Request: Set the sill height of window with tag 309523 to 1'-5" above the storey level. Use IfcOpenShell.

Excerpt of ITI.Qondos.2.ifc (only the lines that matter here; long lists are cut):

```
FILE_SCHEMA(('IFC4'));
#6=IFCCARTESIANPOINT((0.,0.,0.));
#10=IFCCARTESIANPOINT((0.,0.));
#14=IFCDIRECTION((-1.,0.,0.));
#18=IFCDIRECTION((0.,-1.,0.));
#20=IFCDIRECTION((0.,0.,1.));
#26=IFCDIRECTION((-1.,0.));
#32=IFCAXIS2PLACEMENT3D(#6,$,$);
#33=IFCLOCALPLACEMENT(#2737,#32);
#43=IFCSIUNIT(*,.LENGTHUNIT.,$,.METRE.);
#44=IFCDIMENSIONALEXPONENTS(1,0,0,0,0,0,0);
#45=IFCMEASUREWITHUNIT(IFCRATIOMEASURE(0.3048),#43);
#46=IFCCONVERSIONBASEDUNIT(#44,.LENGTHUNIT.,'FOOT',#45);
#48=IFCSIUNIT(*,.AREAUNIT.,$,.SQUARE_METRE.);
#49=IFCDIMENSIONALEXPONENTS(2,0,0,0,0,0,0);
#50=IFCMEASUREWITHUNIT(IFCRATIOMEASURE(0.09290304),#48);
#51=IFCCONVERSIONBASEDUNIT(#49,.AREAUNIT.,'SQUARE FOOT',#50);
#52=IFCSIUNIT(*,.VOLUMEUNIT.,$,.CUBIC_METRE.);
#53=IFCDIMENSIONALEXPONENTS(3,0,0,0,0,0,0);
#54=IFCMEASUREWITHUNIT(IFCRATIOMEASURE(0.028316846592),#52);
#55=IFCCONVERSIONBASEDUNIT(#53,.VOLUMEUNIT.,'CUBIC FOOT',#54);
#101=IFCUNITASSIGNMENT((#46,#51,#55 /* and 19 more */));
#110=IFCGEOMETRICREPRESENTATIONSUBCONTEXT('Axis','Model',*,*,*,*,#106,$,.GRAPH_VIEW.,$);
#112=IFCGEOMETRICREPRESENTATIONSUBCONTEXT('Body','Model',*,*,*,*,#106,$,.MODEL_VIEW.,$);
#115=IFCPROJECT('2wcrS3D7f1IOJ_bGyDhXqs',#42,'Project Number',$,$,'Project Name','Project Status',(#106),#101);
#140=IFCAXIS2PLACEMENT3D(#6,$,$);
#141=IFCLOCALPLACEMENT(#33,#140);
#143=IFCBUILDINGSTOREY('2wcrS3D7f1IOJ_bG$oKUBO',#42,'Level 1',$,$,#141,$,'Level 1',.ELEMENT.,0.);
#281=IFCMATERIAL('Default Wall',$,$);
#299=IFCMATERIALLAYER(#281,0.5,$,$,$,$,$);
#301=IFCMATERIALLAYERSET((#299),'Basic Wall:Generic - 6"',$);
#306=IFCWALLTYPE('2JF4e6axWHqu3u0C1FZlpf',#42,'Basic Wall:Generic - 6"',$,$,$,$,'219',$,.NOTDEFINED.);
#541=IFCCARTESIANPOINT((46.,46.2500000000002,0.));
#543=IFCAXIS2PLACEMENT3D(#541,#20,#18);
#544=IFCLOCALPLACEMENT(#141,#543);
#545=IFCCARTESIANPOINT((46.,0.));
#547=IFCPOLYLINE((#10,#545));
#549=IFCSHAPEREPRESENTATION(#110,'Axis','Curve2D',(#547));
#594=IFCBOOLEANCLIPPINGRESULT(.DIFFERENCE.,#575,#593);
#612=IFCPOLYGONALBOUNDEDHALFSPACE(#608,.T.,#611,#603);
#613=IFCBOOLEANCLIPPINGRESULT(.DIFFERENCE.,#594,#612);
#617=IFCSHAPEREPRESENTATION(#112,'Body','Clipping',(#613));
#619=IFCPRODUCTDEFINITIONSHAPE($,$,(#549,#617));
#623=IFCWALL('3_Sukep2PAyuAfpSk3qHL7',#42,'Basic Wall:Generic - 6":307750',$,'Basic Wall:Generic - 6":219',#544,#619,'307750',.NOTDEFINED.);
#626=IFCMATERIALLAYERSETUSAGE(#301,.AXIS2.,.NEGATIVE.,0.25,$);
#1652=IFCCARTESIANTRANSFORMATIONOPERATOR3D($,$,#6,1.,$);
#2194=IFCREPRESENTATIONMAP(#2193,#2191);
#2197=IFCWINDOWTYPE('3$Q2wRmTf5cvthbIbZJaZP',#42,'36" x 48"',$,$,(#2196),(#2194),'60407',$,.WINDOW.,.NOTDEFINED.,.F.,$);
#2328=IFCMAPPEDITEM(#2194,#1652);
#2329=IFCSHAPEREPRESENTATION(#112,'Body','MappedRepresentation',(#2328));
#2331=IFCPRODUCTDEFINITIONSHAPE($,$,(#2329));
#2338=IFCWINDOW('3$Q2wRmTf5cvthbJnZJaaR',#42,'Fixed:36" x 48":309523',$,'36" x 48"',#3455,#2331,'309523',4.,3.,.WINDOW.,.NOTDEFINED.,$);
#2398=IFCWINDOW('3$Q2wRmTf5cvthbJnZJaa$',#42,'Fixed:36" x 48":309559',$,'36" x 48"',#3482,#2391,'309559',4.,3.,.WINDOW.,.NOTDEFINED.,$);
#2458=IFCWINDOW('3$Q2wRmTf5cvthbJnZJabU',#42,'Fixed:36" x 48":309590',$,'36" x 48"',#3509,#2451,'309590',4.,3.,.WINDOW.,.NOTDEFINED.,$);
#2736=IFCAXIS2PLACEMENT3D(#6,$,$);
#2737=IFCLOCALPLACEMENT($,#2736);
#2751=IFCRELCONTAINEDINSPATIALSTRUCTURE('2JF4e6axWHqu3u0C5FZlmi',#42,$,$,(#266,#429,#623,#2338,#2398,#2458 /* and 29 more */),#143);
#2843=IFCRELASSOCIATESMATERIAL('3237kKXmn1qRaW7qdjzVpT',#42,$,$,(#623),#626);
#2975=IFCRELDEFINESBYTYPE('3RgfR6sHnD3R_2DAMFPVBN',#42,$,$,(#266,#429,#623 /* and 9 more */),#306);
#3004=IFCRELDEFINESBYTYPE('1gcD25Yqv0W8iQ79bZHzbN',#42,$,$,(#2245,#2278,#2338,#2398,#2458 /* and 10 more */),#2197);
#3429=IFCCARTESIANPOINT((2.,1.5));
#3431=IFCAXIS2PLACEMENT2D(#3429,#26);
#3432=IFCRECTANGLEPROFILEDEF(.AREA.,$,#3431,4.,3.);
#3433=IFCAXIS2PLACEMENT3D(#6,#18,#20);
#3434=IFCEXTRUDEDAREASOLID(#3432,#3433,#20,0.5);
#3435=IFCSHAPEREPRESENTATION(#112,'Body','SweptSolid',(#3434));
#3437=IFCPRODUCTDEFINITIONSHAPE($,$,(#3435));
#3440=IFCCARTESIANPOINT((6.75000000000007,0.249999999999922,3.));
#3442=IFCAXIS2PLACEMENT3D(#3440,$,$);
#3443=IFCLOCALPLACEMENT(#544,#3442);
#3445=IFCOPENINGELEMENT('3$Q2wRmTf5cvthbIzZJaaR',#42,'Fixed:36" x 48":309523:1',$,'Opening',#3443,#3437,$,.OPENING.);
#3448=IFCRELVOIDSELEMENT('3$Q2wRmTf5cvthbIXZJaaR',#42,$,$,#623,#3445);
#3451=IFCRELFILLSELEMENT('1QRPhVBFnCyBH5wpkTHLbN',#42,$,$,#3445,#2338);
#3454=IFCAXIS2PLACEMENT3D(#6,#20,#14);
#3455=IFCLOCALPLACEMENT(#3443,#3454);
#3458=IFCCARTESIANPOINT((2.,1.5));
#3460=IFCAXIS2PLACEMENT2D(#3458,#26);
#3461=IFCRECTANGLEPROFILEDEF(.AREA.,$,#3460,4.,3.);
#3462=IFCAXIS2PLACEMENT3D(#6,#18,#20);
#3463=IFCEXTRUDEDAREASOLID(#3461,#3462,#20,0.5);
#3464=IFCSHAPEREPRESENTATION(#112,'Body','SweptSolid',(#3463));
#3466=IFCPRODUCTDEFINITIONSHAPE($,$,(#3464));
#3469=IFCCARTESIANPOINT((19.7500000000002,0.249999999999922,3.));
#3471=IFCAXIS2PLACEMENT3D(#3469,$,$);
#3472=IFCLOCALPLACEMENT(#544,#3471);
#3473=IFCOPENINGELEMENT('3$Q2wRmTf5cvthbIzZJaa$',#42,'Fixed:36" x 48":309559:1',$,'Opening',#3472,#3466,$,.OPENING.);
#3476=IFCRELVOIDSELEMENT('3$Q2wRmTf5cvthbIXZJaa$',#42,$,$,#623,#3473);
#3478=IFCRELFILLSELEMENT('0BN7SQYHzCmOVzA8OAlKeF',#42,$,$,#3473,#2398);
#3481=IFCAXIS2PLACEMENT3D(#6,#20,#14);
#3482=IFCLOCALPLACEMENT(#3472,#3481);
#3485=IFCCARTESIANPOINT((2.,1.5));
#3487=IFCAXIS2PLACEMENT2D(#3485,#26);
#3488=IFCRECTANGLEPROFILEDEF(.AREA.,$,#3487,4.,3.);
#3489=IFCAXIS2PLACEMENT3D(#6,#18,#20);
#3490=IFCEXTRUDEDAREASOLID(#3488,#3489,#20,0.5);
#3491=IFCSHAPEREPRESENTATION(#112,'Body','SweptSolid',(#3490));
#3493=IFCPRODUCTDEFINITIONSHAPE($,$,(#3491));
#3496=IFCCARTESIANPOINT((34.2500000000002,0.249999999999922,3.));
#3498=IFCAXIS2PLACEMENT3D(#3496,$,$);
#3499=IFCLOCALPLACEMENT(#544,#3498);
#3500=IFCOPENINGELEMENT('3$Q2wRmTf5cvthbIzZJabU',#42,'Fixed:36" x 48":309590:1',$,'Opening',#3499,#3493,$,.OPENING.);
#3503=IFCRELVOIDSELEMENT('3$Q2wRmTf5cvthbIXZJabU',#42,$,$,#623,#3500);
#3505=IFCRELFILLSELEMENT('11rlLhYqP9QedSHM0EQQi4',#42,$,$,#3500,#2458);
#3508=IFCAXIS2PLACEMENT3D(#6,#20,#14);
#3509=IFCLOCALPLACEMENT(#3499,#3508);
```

```python
import numpy as np
import ifcopenshell
import ifcopenshell.api.geometry
import ifcopenshell.geom
import ifcopenshell.util.element
import ifcopenshell.util.placement
import ifcopenshell.util.shape
import ifcopenshell.util.unit

model = ifcopenshell.open("ITI.Qondos.2.ifc")
unit_scale = ifcopenshell.util.unit.calculate_unit_scale(model)

window = model.by_guid("3$Q2wRmTf5cvthbJnZJaaR")
opening = window.FillsVoids[0].RelatingOpeningElement
storey = ifcopenshell.util.element.get_container(window, ifc_class="IfcBuildingStorey")
level = ifcopenshell.util.placement.get_local_placement(storey.ObjectPlacement)[2, 3]

# The opening's origin need not be at the sill, so measure its lowest point.
shape = ifcopenshell.geom.create_shape(ifcopenshell.geom.settings(), opening)
bottom = ifcopenshell.util.shape.get_shape_bottom_elevation(shape, shape.geometry) / unit_scale
dz = level + 17 * 0.0254 / unit_scale - bottom

shift = np.array([0.0, 0.0, dz])
# The window is placed relative to its opening, so it follows when the opening moves.
matrix = ifcopenshell.util.placement.get_local_placement(opening.ObjectPlacement)
matrix[:3, 3] += shift
ifcopenshell.api.geometry.edit_object_placement(
    model, product=opening, matrix=matrix, is_si=False, should_transform_children=True
)

print(f"moved by {dz * unit_scale:+.3f} m")

model.write("ITI.Qondos.2_edited.ifc")
```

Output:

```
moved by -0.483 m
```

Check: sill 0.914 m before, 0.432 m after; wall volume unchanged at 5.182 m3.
